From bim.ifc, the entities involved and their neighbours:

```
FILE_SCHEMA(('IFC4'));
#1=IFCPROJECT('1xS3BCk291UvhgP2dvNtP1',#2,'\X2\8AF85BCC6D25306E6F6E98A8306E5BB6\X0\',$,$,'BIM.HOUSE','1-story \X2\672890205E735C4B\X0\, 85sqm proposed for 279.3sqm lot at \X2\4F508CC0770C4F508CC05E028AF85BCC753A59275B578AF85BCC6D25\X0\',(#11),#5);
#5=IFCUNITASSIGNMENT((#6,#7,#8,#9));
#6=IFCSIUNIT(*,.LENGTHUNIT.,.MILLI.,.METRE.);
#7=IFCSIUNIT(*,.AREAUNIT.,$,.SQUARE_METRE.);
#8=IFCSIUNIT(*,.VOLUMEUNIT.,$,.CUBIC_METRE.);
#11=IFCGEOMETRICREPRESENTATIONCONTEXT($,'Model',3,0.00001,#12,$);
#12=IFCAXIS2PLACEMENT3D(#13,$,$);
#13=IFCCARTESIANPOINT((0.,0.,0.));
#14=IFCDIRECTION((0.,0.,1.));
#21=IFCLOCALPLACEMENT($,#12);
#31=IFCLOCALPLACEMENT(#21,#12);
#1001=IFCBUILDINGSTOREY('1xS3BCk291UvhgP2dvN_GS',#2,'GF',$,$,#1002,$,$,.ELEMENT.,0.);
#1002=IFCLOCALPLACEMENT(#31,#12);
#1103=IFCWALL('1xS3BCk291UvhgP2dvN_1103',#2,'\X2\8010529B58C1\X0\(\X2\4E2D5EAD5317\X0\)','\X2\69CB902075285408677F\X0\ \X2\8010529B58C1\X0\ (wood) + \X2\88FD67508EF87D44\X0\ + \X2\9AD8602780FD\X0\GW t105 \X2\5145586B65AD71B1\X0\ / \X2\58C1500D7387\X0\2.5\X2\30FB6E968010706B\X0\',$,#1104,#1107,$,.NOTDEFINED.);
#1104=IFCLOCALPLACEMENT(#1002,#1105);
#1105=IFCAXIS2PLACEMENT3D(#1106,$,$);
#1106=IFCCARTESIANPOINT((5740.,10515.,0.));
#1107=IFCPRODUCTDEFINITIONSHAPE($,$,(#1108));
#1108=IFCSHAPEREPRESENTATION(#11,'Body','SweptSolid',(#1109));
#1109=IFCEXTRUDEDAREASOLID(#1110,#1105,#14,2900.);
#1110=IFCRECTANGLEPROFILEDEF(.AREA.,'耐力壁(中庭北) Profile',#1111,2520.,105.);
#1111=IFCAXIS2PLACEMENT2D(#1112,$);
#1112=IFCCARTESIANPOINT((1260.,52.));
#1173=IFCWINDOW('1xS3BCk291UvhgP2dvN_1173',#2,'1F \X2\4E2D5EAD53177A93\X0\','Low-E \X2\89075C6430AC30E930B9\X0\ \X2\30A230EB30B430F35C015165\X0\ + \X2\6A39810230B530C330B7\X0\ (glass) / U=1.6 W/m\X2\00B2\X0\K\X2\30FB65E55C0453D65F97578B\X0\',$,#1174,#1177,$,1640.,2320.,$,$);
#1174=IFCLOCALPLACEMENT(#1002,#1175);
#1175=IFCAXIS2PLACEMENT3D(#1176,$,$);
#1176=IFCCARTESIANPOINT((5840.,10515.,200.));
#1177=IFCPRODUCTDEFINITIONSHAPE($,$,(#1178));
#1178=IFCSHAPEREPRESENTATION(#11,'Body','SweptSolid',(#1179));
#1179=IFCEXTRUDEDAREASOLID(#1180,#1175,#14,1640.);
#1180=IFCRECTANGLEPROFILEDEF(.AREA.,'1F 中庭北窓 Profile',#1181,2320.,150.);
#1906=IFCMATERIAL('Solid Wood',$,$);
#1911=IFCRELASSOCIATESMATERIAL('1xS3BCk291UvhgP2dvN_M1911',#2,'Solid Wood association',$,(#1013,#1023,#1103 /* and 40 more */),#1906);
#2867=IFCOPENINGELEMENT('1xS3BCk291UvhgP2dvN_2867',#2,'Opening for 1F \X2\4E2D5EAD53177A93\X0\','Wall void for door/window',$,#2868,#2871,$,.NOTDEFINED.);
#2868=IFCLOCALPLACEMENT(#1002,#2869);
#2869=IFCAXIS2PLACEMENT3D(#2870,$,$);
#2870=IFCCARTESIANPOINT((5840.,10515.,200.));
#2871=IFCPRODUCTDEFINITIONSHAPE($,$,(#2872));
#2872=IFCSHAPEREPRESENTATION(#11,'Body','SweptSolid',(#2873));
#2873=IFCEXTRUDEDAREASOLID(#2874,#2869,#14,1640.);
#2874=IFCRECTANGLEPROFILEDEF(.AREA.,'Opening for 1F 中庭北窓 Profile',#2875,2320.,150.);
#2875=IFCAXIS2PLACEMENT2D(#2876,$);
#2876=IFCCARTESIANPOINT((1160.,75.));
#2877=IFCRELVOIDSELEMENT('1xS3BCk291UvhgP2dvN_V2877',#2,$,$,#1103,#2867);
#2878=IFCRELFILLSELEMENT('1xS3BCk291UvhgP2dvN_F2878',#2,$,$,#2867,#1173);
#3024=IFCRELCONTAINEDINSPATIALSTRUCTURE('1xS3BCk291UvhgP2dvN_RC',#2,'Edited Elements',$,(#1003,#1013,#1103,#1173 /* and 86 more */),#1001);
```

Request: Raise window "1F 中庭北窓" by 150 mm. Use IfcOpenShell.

```python
import numpy as np
import ifcopenshell
import ifcopenshell.api.geometry
import ifcopenshell.util.placement
import ifcopenshell.util.unit

model = ifcopenshell.open("bim.ifc")
unit_scale = ifcopenshell.util.unit.calculate_unit_scale(model)

window = model.by_guid("1xS3BCk291UvhgP2dvN_1173")
opening = window.FillsVoids[0].RelatingOpeningElement
dz = 0.15 / unit_scale

shift = np.array([0.0, 0.0, dz])
# The window is not placed relative to its opening, so move both.
for product in (opening, window):
    matrix = ifcopenshell.util.placement.get_local_placement(product.ObjectPlacement)
    matrix[:3, 3] += shift
    ifcopenshell.api.geometry.edit_object_placement(model, product=product, matrix=matrix, is_si=False)

print(f"moved by {dz * unit_scale:+.3f} m")

model.write("bim-out.ifc")
```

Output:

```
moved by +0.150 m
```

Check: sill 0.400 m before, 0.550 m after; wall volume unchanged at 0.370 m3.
